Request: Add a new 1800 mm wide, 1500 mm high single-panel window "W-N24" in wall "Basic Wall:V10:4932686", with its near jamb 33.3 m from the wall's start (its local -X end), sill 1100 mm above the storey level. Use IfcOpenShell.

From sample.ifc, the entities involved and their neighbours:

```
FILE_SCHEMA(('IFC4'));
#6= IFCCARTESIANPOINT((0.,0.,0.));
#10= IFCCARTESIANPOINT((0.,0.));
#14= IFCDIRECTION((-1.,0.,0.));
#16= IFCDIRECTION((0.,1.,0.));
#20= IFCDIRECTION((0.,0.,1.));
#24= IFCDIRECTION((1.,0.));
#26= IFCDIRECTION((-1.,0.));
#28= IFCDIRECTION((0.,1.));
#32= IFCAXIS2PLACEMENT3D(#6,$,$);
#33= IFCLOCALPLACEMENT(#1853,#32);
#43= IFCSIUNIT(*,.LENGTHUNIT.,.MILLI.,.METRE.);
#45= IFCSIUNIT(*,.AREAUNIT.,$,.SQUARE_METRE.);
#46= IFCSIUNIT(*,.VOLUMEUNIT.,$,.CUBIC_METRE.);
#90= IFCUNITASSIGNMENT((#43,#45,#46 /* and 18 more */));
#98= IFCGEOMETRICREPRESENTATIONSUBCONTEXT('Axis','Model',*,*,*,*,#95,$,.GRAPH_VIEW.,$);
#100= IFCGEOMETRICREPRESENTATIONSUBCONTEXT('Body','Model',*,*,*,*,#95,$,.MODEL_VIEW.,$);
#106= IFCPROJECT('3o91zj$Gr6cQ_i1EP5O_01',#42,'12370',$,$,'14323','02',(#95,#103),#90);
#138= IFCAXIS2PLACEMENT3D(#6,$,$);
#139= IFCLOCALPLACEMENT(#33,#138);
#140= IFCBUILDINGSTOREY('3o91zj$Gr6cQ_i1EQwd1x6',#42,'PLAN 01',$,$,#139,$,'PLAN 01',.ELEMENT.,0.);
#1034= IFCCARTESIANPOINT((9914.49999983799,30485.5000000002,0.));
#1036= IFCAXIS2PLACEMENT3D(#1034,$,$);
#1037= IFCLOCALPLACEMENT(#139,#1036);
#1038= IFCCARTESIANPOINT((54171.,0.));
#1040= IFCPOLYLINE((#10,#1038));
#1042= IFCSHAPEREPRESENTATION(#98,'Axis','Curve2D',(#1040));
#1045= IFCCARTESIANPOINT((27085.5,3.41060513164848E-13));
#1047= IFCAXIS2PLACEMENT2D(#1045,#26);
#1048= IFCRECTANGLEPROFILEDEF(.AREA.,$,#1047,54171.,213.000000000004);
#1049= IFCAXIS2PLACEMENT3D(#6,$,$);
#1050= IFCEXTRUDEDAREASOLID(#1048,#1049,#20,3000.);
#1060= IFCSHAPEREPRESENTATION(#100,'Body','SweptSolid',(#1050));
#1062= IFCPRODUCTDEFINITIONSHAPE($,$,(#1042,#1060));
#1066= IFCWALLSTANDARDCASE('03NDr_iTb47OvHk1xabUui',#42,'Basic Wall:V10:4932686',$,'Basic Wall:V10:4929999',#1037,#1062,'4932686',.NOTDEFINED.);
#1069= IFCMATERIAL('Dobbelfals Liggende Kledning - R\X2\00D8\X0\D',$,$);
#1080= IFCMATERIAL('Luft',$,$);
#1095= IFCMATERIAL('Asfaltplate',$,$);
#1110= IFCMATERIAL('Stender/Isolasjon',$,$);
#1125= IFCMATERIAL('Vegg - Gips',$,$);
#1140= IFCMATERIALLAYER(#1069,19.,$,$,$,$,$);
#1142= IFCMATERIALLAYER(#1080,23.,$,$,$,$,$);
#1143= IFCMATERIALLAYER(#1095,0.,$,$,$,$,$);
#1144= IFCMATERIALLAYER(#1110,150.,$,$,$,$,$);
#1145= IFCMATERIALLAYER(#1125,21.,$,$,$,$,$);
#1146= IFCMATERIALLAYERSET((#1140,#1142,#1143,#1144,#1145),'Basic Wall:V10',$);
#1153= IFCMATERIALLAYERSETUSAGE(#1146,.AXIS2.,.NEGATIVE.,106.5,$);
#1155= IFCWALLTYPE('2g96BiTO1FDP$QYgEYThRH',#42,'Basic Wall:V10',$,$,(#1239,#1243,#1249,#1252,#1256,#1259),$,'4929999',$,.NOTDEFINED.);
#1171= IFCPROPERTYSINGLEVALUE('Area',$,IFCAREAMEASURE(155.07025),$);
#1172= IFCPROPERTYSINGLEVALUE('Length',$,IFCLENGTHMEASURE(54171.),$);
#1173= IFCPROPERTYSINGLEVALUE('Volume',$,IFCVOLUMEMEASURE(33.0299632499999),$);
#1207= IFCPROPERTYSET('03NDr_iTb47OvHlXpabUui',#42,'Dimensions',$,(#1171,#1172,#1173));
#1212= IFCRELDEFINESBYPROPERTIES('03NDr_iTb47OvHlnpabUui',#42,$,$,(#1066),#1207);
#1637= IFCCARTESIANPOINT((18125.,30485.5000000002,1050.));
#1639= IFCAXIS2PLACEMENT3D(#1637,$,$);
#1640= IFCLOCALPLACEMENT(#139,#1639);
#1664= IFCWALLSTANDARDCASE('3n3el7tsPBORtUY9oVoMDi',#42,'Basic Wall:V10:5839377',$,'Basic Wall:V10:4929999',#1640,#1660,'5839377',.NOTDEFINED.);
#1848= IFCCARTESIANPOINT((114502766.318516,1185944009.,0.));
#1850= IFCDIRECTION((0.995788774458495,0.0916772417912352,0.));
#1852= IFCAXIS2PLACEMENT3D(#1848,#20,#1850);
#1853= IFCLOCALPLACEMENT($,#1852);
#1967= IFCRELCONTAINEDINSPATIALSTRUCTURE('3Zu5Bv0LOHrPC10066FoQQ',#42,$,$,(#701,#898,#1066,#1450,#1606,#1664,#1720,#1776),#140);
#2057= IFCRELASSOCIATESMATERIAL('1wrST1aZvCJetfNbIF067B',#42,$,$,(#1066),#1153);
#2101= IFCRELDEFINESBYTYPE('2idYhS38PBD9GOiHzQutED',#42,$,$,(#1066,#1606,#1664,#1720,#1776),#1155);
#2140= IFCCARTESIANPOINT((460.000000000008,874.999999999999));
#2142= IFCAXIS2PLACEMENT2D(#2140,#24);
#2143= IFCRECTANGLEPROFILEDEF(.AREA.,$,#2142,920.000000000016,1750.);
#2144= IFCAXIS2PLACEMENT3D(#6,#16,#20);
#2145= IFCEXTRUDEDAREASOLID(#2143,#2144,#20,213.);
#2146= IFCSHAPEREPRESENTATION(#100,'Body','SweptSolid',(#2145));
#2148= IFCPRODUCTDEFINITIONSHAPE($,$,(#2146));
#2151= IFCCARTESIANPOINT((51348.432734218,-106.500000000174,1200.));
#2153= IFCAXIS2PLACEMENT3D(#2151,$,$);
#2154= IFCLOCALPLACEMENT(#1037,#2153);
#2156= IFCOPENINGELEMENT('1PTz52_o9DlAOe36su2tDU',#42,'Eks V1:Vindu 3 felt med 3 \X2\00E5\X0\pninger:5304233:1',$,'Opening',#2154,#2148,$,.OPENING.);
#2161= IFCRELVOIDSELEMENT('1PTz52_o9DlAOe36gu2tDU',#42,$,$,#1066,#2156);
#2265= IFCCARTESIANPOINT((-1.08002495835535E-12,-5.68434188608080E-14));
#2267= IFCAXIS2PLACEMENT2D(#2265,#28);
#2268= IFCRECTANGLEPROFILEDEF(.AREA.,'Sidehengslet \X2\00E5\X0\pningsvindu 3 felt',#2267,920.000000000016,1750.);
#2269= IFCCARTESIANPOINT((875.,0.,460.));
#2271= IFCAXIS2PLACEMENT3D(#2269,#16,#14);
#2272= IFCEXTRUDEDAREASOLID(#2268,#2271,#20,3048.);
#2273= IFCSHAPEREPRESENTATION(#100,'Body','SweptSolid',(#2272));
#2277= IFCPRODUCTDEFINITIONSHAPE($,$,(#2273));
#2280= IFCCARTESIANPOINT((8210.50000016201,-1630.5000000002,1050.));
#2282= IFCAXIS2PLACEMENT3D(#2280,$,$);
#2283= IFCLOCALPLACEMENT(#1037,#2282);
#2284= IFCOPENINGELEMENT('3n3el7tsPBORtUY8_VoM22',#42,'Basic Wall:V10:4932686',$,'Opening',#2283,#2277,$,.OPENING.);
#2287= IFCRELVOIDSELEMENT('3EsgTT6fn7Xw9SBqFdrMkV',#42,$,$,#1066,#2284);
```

```python
import numpy as np
import ifcopenshell
import ifcopenshell.api.feature
import ifcopenshell.api.geometry
import ifcopenshell.api.pset
import ifcopenshell.api.root
import ifcopenshell.api.spatial
import ifcopenshell.geom
import ifcopenshell.util.element
import ifcopenshell.util.placement
import ifcopenshell.util.representation
import ifcopenshell.util.shape
import ifcopenshell.util.unit

model = ifcopenshell.open("sample.ifc")
unit_scale = ifcopenshell.util.unit.calculate_unit_scale(model)
area_scale = ifcopenshell.util.unit.calculate_unit_scale(model, "AREAUNIT")
volume_scale = ifcopenshell.util.unit.calculate_unit_scale(model, "VOLUMEUNIT")
settings = ifcopenshell.geom.settings()


def volume(element):
    """Net volume in cubic metres, openings subtracted."""
    shape = ifcopenshell.geom.create_shape(settings, element)
    return ifcopenshell.util.shape.get_volume(shape.geometry)


wall = model.by_guid("03NDr_iTb47OvHk1xabUui")
storey = ifcopenshell.util.element.get_container(wall, ifc_class="IfcBuildingStorey")
context = ifcopenshell.util.representation.get_context(model, "Model", "Body", "MODEL_VIEW")
before = volume(wall)

width, height, from_end, sill = 1.8, 1.5, 33.3, 1.1  # metres

# The wall runs along its own X axis, and the end named is its -X end.
wall_shape = ifcopenshell.geom.create_shape(settings, wall)
x, y, z = ifcopenshell.util.shape.get_vertices(wall_shape.geometry).T
start = x.min() + from_end
face, thickness = float(y.min()), float(y.max() - y.min())
wall_matrix = ifcopenshell.util.placement.get_local_placement(wall.ObjectPlacement)
level = ifcopenshell.util.placement.get_local_placement(storey.ObjectPlacement)[2, 3]


def in_wall(x, y):
    """Placement at x, y metres in the wall's axes, at sill height."""
    matrix = wall_matrix.copy()
    matrix[:, 3] = wall_matrix @ np.array([x / unit_scale, y / unit_scale, 0.0, 1.0])
    matrix[2, 3] = level + sill / unit_scale
    return matrix


# Opening: a box that overshoots both wall faces by 50 mm.
opening = ifcopenshell.api.root.create_entity(model, ifc_class="IfcOpeningElement", predefined_type="OPENING")
box = ifcopenshell.api.geometry.add_wall_representation(
    model, context=context, length=width, height=height, thickness=thickness + 0.1
)
ifcopenshell.api.geometry.assign_representation(model, product=opening, representation=box)
ifcopenshell.api.geometry.edit_object_placement(model, product=opening, matrix=in_wall(start, face - 0.05), is_si=False)
ifcopenshell.api.feature.add_feature(model, feature=opening, element=wall)

window = ifcopenshell.api.root.create_entity(model, ifc_class="IfcWindow", name="W-N24", predefined_type="WINDOW")
window.OverallWidth, window.OverallHeight = width / unit_scale, height / unit_scale
window.PartitioningType = "SINGLE_PANEL"
body = ifcopenshell.api.geometry.add_window_representation(
    model,
    context=context,
    overall_width=window.OverallWidth,
    overall_height=window.OverallHeight,
    partition_type="SINGLE_PANEL",
)
ifcopenshell.api.geometry.assign_representation(model, product=window, representation=body)
ifcopenshell.api.spatial.assign_container(model, products=[window], relating_structure=storey)
ifcopenshell.api.feature.add_filling(model, opening=opening, element=window)

# Centre the window in the wall's thickness.
ifcopenshell.api.geometry.edit_object_placement(model, product=window, matrix=in_wall(start, face), is_si=False)
window_shape = ifcopenshell.geom.create_shape(settings, window)
depth = ifcopenshell.util.shape.get_vertices(window_shape.geometry)[:, 1]
offset = face + thickness / 2 - (depth.min() + depth.max()) / 2
ifcopenshell.api.geometry.edit_object_placement(model, product=window, matrix=in_wall(start, offset), is_si=False)

after = volume(wall)

# Update the wall's stored quantities.
pset = model.by_id(ifcopenshell.util.element.get_pset(wall, "Dimensions", should_inherit=False)["id"])
ifcopenshell.api.pset.edit_pset(model, pset=pset, properties={
    "Area": model.create_entity("IfcAreaMeasure", after / thickness / area_scale),
    "Volume": model.create_entity("IfcVolumeMeasure", after / volume_scale),
})

print(f"wall volume {before:.3f} -> {after:.3f} m3")

model.write("sample-out.ifc")
```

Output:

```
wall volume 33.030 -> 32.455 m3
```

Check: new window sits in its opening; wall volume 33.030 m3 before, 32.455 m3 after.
